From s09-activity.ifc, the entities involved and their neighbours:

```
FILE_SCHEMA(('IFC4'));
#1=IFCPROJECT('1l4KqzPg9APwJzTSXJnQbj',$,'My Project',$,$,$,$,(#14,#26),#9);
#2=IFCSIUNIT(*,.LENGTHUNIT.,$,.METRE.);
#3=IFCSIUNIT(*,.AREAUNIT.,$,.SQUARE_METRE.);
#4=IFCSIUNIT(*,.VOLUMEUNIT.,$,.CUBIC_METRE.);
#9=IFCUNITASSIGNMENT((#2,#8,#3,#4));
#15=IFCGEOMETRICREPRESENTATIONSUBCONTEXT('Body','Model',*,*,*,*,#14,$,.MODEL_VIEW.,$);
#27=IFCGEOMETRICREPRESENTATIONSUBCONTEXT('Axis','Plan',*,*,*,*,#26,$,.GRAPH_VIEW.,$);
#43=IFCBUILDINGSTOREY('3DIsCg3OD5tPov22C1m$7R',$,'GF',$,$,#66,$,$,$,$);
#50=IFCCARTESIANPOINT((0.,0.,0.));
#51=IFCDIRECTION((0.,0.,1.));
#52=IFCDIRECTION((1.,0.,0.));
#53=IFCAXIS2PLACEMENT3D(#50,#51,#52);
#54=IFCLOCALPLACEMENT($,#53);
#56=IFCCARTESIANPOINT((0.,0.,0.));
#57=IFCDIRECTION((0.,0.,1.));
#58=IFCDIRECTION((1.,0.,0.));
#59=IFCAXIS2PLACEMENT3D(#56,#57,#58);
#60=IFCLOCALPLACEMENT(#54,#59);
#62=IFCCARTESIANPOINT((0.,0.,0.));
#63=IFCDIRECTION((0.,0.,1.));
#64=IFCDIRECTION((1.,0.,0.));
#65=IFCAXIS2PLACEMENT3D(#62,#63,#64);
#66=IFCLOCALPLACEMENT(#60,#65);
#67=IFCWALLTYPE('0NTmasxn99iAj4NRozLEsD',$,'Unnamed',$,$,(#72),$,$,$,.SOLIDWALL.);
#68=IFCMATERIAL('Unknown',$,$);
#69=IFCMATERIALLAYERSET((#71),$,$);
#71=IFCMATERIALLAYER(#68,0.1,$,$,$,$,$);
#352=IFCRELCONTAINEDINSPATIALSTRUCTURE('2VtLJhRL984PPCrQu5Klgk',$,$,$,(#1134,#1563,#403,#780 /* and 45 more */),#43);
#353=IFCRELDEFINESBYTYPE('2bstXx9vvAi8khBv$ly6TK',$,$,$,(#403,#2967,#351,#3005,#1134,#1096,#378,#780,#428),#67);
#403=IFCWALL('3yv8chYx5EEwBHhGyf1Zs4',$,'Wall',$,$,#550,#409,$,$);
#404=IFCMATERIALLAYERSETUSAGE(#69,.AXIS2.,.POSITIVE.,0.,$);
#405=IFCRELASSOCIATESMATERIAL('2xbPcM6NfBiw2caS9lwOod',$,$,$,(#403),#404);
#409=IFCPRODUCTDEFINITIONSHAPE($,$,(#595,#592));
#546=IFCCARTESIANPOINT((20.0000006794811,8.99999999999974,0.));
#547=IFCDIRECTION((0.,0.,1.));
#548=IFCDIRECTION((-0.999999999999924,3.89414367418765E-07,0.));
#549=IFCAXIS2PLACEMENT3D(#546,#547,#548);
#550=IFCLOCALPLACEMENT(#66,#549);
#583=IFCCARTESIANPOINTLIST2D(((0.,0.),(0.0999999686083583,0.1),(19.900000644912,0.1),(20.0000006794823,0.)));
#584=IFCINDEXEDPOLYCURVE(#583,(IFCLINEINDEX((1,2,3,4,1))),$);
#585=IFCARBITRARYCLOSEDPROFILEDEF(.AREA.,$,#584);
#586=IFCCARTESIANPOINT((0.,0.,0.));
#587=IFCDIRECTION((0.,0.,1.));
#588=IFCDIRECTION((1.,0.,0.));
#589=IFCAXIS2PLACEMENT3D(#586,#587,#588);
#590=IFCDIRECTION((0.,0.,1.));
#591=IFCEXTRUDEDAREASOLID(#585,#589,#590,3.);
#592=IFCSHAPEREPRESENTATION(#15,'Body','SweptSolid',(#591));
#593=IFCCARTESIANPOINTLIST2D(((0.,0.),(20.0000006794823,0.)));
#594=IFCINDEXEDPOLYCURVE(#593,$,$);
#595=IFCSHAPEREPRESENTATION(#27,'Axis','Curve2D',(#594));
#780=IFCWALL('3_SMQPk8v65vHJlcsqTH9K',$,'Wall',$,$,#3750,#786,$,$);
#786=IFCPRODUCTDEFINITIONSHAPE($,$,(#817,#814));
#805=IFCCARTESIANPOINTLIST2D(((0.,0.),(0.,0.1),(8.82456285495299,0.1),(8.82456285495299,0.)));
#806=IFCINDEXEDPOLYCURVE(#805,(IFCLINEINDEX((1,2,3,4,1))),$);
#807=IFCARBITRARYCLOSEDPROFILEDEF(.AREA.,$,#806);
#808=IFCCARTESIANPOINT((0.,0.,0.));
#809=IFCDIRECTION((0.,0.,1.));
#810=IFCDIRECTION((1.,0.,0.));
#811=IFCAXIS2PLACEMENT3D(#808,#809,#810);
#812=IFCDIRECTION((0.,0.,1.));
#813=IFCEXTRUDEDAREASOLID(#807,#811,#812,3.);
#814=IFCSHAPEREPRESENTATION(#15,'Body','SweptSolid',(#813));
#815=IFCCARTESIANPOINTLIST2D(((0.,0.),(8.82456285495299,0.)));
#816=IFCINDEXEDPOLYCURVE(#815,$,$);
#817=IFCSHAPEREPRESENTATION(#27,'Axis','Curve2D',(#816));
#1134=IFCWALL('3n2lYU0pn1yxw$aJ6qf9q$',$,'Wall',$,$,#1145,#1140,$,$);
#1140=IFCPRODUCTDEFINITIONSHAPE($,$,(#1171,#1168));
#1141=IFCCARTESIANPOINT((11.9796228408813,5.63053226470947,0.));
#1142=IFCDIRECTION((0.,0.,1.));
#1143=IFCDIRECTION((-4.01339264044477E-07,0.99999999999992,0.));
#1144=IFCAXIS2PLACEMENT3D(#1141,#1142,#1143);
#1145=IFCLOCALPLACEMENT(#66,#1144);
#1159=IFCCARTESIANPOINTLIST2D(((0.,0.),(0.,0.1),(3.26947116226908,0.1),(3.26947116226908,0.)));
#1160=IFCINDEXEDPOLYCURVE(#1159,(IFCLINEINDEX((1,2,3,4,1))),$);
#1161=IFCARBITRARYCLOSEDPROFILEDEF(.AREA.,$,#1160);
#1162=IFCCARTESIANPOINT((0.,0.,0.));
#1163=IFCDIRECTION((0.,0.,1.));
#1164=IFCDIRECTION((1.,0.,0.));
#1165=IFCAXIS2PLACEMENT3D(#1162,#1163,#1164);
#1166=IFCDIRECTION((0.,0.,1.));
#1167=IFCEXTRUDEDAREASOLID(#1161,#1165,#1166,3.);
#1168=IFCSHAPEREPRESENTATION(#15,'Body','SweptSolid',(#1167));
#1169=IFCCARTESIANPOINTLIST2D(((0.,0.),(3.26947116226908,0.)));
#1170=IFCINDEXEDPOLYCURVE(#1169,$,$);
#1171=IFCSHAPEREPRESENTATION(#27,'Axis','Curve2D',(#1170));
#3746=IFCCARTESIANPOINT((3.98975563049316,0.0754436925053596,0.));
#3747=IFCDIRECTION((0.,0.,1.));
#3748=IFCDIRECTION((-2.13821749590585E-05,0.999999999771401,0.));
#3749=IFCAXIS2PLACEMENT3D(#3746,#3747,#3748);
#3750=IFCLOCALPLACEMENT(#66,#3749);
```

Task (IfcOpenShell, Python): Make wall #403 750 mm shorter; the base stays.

```python
import ifcopenshell
import ifcopenshell.geom
import ifcopenshell.util.representation
import ifcopenshell.util.shape
import ifcopenshell.util.unit

model = ifcopenshell.open("s09-activity.ifc")
unit_scale = ifcopenshell.util.unit.calculate_unit_scale(model)
settings = ifcopenshell.geom.settings()


def volume(element):
    """Net volume in cubic metres, openings subtracted."""
    shape = ifcopenshell.geom.create_shape(settings, element)
    return ifcopenshell.util.shape.get_volume(shape.geometry)


wall = model.by_id(403)
before = volume(wall)

body = ifcopenshell.util.representation.get_representation(wall, "Model", "Body")
solid = body.Items[0]
old_height = solid.Depth
solid.Depth -= 0.75 / unit_scale
after = volume(wall)

print(f"height {old_height:g} -> {solid.Depth:g}, volume {before:.3f} -> {after:.3f} m3")

model.write("s09-activity_rev.ifc")
```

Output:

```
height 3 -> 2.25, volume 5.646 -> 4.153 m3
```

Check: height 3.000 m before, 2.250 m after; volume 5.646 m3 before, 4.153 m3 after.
